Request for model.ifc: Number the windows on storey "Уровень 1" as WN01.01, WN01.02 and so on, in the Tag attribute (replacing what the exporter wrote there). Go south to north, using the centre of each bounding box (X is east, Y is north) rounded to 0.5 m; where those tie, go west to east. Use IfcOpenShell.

First a look at what the model holds.

```python
import ifcopenshell
import ifcopenshell.util.element
import ifcopenshell.util.placement

model = ifcopenshell.open("model.ifc")
print(model.schema)
storey = next(s for s in model.by_type("IfcBuildingStorey") if s.Name == "Уровень 1")
windows = [e for e in ifcopenshell.util.element.get_decomposition(storey) if e.is_a("IfcWindow")]
for e in sorted(windows, key=lambda e: e.id()):
    origin = ifcopenshell.util.placement.get_local_placement(e.ObjectPlacement)[:3, 3]
    print(e.id(), e.Tag, e.Name, origin.round(2) + 0.0, sep=" | ")
```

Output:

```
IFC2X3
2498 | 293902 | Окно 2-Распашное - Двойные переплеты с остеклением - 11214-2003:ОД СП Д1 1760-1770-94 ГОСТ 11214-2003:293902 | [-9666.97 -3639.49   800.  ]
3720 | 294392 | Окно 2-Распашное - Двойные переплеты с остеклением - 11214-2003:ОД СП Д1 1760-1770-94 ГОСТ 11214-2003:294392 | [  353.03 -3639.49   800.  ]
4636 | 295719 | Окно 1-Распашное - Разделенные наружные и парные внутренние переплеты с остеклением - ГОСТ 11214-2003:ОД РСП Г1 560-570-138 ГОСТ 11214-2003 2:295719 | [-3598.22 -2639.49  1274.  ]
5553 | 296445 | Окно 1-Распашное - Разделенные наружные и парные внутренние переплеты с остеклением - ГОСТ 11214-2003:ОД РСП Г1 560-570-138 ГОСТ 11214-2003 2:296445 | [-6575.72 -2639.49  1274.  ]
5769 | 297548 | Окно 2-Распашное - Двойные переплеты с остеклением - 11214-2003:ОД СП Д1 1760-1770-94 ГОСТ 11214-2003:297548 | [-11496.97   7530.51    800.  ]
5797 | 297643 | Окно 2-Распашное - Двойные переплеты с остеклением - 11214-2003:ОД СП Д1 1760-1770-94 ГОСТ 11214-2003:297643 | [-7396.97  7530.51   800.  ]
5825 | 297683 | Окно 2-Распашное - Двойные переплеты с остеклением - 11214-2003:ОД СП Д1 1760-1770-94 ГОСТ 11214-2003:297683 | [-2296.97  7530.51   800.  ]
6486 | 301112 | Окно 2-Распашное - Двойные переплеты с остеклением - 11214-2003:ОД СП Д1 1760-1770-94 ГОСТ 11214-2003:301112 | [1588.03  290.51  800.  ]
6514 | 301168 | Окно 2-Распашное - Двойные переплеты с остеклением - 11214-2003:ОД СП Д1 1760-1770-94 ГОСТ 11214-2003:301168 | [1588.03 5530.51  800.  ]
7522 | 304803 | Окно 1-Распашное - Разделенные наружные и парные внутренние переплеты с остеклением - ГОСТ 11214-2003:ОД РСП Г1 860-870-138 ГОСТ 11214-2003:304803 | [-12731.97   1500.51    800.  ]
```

```python
import ifcopenshell
import ifcopenshell.geom
import ifcopenshell.util.element
import ifcopenshell.util.shape

model = ifcopenshell.open("model.ifc")
settings = ifcopenshell.geom.settings()
settings.set("use-world-coords", True)


def centre(element):
    shape = ifcopenshell.geom.create_shape(settings, element)
    return ifcopenshell.util.shape.get_bbox_centroid(shape.geometry)


storey = next(s for s in model.by_type("IfcBuildingStorey") if s.Name == "Уровень 1")
windows = [e for e in ifcopenshell.util.element.get_decomposition(storey) if e.is_a("IfcWindow")]

# Insertion points can sit at a corner or the storey origin, so sort by the geometry (in metres).
centres = {e: centre(e) for e in windows}
windows.sort(key=lambda e: (round(centres[e][1] / 0.5), centres[e][0]))

for i, e in enumerate(windows, start=1):
    number = f"WN01.{i:02d}"
    e.Tag = number
    print(e.id(), number)

model.write("model_rev.ifc")
```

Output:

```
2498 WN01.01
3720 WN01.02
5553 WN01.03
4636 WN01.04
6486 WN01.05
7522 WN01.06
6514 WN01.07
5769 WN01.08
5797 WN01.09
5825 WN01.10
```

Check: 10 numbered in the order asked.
